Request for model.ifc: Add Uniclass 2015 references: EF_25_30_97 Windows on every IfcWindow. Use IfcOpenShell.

First a look at what the model holds.

```python
import ifcopenshell

model = ifcopenshell.open("model.ifc")
print(model.schema)
print("classifications:", [c.Name for c in model.by_type("IfcClassification")])
for ifc_class in ("IfcDoor", "IfcRoof", "IfcStair", "IfcWall", "IfcWindow"):
    print(ifc_class, len(model.by_type(ifc_class)))
```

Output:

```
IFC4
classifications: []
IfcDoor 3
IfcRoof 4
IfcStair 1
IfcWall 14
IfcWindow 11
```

```python
import ifcopenshell
import ifcopenshell.api.classification

model = ifcopenshell.open("model.ifc")

system = ifcopenshell.api.classification.add_classification(model, classification="Uniclass 2015")

codes = {
    "IfcWindow": ("EF_25_30_97", "Windows"),
}
for ifc_class, (code, name) in codes.items():
    products = model.by_type(ifc_class)
    ifcopenshell.api.classification.add_reference(
        model, products=products, classification=system, identification=code, name=name
    )
    print(code, len(products))

model.write("model_updated.ifc")
```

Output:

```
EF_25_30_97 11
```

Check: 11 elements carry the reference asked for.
